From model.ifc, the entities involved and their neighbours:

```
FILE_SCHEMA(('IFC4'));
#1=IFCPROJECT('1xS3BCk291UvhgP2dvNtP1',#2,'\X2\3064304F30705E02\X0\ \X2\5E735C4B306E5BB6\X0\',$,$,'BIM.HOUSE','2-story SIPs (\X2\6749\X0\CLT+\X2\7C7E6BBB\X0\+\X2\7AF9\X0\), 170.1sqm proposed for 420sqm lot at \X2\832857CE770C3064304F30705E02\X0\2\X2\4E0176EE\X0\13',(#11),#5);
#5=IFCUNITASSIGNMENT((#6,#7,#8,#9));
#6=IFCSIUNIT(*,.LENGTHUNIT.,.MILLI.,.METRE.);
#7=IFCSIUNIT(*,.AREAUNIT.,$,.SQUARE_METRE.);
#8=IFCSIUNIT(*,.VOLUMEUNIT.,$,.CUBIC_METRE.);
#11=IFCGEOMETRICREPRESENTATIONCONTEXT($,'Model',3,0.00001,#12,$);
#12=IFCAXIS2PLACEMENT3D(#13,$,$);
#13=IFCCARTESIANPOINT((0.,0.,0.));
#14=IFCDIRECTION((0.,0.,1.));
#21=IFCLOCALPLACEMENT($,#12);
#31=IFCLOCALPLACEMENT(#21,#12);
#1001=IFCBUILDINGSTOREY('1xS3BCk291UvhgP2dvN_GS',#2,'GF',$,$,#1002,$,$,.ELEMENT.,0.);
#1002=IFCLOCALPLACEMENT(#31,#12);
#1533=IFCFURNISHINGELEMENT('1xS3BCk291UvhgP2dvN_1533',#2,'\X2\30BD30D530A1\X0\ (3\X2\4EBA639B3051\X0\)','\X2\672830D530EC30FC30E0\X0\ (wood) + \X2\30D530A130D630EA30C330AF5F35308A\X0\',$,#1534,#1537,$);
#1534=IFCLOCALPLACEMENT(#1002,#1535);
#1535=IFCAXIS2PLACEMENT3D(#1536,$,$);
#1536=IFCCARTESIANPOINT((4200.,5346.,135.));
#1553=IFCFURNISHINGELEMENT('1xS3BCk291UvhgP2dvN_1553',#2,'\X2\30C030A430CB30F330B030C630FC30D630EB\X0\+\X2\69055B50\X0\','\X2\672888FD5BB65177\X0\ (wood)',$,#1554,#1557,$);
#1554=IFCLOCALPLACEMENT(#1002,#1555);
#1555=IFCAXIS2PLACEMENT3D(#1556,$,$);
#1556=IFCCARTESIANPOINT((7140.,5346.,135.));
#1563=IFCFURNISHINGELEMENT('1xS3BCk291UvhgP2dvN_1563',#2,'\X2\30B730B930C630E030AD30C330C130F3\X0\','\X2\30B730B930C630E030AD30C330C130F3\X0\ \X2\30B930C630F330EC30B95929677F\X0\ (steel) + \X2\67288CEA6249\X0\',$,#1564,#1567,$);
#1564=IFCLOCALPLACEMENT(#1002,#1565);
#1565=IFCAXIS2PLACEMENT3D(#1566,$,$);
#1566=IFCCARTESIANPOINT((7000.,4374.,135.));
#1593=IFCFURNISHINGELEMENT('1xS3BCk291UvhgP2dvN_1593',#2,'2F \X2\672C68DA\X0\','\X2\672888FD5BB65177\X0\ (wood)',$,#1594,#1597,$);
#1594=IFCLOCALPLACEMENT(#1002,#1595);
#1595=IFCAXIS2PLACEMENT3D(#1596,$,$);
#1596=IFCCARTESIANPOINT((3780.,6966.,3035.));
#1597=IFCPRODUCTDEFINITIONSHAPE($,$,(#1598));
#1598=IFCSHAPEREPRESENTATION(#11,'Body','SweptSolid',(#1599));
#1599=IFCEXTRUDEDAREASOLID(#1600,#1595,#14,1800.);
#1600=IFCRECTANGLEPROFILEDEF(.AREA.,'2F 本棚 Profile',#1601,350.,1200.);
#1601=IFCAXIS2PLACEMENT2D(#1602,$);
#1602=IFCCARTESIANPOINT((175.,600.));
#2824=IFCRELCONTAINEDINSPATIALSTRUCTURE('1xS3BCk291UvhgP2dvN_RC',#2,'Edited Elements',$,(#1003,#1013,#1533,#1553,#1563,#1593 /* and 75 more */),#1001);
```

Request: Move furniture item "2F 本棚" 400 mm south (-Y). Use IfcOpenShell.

```python
import ifcopenshell
import ifcopenshell.api.geometry
import ifcopenshell.util.placement

model = ifcopenshell.open("model.ifc")

item = model.by_guid("1xS3BCk291UvhgP2dvN_1593")
matrix = ifcopenshell.util.placement.get_local_placement(item.ObjectPlacement)
matrix[1, 3] -= 400.0
ifcopenshell.api.geometry.edit_object_placement(model, product=item, matrix=matrix, is_si=False)

print(ifcopenshell.util.placement.get_local_placement(item.ObjectPlacement).round(3) + 0.0)

model.write("model_v2.ifc")
```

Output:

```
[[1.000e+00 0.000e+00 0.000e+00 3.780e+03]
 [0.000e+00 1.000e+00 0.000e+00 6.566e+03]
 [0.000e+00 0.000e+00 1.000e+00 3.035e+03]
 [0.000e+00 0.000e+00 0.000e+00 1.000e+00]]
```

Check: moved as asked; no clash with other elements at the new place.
